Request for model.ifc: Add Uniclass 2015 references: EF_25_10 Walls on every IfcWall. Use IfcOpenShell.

First a look at what the model holds.

```python
import ifcopenshell

model = ifcopenshell.open("model.ifc")
print(model.schema)
print("classifications:", [c.Name for c in model.by_type("IfcClassification")])
for ifc_class in ("IfcDoor", "IfcRoof", "IfcStair", "IfcWall", "IfcWindow"):
    print(ifc_class, len(model.by_type(ifc_class)))
```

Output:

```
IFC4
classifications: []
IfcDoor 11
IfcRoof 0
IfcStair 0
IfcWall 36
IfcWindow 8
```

```python
import ifcopenshell
import ifcopenshell.api.classification

model = ifcopenshell.open("model.ifc")

system = ifcopenshell.api.classification.add_classification(model, classification="Uniclass 2015")

codes = {
    "IfcWall": ("EF_25_10", "Walls"),
}
for ifc_class, (code, name) in codes.items():
    products = model.by_type(ifc_class)
    ifcopenshell.api.classification.add_reference(
        model, products=products, classification=system, identification=code, name=name
    )
    print(code, len(products))

model.write("model_rev.ifc")
```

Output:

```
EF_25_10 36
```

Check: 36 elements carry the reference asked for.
